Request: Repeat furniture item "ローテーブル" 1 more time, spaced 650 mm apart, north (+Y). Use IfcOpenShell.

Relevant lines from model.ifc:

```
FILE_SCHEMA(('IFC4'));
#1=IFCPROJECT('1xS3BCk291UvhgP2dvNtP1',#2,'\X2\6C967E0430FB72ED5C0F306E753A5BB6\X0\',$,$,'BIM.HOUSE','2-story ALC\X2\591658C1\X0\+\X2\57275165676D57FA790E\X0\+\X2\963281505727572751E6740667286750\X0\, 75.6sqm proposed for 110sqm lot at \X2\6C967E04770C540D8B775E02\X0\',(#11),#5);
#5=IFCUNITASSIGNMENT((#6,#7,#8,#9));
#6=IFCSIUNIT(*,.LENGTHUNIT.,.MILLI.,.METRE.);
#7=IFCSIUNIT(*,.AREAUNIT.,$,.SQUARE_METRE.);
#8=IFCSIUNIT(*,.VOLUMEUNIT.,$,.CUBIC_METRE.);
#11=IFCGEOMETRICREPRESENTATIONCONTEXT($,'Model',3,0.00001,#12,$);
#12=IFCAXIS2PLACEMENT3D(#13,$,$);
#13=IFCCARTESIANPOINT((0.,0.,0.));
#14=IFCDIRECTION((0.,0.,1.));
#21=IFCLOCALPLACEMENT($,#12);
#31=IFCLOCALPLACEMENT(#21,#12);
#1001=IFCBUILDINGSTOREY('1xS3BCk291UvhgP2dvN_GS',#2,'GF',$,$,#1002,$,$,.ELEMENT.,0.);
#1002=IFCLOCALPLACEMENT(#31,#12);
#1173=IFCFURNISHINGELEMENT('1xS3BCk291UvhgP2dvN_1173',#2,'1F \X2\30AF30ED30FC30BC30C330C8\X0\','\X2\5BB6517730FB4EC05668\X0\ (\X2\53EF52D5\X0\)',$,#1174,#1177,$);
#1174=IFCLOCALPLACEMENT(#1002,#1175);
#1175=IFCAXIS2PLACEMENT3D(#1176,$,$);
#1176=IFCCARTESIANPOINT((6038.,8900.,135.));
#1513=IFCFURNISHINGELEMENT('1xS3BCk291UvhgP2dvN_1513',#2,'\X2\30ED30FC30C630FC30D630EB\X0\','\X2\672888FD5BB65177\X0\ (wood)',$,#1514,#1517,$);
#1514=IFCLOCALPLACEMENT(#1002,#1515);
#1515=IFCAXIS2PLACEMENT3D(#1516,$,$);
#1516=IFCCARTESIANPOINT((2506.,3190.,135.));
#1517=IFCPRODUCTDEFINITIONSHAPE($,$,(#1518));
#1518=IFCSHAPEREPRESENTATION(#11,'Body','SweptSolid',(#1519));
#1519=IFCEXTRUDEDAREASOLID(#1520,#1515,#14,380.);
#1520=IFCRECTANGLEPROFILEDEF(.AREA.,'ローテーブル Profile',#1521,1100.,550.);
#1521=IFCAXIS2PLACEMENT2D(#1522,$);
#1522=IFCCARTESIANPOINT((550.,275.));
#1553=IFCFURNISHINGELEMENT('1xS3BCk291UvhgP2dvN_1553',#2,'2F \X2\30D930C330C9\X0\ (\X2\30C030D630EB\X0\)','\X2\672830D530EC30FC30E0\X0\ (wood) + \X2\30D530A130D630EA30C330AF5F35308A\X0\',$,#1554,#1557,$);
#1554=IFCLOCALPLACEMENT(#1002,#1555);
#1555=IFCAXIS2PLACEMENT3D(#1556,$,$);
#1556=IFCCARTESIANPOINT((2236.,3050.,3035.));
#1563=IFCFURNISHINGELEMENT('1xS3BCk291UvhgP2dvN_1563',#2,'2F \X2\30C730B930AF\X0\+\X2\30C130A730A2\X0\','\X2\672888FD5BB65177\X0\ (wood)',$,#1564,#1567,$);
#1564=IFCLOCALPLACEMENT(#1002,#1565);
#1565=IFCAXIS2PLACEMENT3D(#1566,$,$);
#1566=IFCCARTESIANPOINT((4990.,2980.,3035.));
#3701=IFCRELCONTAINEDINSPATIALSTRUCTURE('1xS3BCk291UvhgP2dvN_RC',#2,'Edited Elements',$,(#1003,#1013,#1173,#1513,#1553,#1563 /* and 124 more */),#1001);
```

```python
import numpy as np
import ifcopenshell
import ifcopenshell.api.geometry
import ifcopenshell.api.root
import ifcopenshell.util.element
import ifcopenshell.util.placement
import ifcopenshell.util.unit

model = ifcopenshell.open("model.ifc")
unit_scale = ifcopenshell.util.unit.calculate_unit_scale(model)


def reuse_history(source, copy):
    """copy_class also copies each property set's owner history, people and application; keep the originals."""
    for rel in copy.IsDefinedBy:
        if rel.is_a("IfcRelDefinesByProperties") and (history := rel.RelatingPropertyDefinition.OwnerHistory):
            rel.RelatingPropertyDefinition.OwnerHistory = source.OwnerHistory
            ifcopenshell.util.element.remove_deep2(model, history)


source = model.by_id(1513)
base = ifcopenshell.util.placement.get_local_placement(source.ObjectPlacement)
step = np.array([0.0, 1.0, 0.0]) * 0.65 / unit_scale

for i in range(1, 2):
    copy = ifcopenshell.api.root.copy_class(model, product=source)
    copy.Representation = ifcopenshell.util.element.copy_deep(
        model, source.Representation, exclude=["IfcGeometricRepresentationContext", "IfcRepresentationMap"]
    )
    reuse_history(source, copy)
    matrix = base.copy()
    matrix[:3, 3] += i * step
    print("added at", matrix[:3, 3].round(3) + 0.0)
    ifcopenshell.api.geometry.edit_object_placement(model, product=copy, matrix=matrix, is_si=False)

model.write("model_updated.ifc")
```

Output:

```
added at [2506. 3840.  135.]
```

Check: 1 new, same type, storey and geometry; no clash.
